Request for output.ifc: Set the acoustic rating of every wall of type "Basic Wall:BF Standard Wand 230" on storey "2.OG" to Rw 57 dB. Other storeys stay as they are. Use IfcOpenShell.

First a look at what the model holds.

```python
import ifcopenshell
import ifcopenshell.util.element

model = ifcopenshell.open("output.ifc")
print(model.schema)
storey = next(s for s in model.by_type("IfcBuildingStorey") if s.Name == "2.OG")
walls = [e for e in ifcopenshell.util.element.get_decomposition(storey) if e.is_a("IfcWall")]
seen = {}
for e in walls:
    element_type = ifcopenshell.util.element.get_type(e)
    key = (element_type.Name if element_type != e and element_type else None, ifcopenshell.util.element.get_pset(e, "Pset_WallCommon", "AcousticRating"))
    seen[key] = seen.get(key, 0) + 1
for (name, value), count in sorted(seen.items(), key=str):
    print(count, "x", name, "|", value)
```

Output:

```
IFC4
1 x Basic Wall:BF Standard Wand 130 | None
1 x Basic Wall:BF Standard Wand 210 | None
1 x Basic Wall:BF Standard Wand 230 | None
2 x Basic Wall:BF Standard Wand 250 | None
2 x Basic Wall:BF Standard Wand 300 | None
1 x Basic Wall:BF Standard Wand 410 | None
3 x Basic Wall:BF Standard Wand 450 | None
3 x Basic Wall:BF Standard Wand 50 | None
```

```python
import ifcopenshell
import ifcopenshell.api.pset
import ifcopenshell.util.element

model = ifcopenshell.open("output.ifc")

storey = next(s for s in model.by_type("IfcBuildingStorey") if s.Name == "2.OG")
walls = [e for e in ifcopenshell.util.element.get_decomposition(storey) if e.is_a("IfcWall")]

count = 0
for e in walls:
    element_type = ifcopenshell.util.element.get_type(e)
    if element_type in (None, e) or element_type.Name != "Basic Wall:BF Standard Wand 230":
        continue
    # add_pset returns the element's existing set when there is one.
    pset = ifcopenshell.api.pset.add_pset(model, product=e, name="Pset_WallCommon")
    ifcopenshell.api.pset.edit_pset(model, pset=pset, properties={"AcousticRating": "Rw 57 dB"})
    count += 1

print(count, "walls updated")

model.write("output_v2.ifc")
```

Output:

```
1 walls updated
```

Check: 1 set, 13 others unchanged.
